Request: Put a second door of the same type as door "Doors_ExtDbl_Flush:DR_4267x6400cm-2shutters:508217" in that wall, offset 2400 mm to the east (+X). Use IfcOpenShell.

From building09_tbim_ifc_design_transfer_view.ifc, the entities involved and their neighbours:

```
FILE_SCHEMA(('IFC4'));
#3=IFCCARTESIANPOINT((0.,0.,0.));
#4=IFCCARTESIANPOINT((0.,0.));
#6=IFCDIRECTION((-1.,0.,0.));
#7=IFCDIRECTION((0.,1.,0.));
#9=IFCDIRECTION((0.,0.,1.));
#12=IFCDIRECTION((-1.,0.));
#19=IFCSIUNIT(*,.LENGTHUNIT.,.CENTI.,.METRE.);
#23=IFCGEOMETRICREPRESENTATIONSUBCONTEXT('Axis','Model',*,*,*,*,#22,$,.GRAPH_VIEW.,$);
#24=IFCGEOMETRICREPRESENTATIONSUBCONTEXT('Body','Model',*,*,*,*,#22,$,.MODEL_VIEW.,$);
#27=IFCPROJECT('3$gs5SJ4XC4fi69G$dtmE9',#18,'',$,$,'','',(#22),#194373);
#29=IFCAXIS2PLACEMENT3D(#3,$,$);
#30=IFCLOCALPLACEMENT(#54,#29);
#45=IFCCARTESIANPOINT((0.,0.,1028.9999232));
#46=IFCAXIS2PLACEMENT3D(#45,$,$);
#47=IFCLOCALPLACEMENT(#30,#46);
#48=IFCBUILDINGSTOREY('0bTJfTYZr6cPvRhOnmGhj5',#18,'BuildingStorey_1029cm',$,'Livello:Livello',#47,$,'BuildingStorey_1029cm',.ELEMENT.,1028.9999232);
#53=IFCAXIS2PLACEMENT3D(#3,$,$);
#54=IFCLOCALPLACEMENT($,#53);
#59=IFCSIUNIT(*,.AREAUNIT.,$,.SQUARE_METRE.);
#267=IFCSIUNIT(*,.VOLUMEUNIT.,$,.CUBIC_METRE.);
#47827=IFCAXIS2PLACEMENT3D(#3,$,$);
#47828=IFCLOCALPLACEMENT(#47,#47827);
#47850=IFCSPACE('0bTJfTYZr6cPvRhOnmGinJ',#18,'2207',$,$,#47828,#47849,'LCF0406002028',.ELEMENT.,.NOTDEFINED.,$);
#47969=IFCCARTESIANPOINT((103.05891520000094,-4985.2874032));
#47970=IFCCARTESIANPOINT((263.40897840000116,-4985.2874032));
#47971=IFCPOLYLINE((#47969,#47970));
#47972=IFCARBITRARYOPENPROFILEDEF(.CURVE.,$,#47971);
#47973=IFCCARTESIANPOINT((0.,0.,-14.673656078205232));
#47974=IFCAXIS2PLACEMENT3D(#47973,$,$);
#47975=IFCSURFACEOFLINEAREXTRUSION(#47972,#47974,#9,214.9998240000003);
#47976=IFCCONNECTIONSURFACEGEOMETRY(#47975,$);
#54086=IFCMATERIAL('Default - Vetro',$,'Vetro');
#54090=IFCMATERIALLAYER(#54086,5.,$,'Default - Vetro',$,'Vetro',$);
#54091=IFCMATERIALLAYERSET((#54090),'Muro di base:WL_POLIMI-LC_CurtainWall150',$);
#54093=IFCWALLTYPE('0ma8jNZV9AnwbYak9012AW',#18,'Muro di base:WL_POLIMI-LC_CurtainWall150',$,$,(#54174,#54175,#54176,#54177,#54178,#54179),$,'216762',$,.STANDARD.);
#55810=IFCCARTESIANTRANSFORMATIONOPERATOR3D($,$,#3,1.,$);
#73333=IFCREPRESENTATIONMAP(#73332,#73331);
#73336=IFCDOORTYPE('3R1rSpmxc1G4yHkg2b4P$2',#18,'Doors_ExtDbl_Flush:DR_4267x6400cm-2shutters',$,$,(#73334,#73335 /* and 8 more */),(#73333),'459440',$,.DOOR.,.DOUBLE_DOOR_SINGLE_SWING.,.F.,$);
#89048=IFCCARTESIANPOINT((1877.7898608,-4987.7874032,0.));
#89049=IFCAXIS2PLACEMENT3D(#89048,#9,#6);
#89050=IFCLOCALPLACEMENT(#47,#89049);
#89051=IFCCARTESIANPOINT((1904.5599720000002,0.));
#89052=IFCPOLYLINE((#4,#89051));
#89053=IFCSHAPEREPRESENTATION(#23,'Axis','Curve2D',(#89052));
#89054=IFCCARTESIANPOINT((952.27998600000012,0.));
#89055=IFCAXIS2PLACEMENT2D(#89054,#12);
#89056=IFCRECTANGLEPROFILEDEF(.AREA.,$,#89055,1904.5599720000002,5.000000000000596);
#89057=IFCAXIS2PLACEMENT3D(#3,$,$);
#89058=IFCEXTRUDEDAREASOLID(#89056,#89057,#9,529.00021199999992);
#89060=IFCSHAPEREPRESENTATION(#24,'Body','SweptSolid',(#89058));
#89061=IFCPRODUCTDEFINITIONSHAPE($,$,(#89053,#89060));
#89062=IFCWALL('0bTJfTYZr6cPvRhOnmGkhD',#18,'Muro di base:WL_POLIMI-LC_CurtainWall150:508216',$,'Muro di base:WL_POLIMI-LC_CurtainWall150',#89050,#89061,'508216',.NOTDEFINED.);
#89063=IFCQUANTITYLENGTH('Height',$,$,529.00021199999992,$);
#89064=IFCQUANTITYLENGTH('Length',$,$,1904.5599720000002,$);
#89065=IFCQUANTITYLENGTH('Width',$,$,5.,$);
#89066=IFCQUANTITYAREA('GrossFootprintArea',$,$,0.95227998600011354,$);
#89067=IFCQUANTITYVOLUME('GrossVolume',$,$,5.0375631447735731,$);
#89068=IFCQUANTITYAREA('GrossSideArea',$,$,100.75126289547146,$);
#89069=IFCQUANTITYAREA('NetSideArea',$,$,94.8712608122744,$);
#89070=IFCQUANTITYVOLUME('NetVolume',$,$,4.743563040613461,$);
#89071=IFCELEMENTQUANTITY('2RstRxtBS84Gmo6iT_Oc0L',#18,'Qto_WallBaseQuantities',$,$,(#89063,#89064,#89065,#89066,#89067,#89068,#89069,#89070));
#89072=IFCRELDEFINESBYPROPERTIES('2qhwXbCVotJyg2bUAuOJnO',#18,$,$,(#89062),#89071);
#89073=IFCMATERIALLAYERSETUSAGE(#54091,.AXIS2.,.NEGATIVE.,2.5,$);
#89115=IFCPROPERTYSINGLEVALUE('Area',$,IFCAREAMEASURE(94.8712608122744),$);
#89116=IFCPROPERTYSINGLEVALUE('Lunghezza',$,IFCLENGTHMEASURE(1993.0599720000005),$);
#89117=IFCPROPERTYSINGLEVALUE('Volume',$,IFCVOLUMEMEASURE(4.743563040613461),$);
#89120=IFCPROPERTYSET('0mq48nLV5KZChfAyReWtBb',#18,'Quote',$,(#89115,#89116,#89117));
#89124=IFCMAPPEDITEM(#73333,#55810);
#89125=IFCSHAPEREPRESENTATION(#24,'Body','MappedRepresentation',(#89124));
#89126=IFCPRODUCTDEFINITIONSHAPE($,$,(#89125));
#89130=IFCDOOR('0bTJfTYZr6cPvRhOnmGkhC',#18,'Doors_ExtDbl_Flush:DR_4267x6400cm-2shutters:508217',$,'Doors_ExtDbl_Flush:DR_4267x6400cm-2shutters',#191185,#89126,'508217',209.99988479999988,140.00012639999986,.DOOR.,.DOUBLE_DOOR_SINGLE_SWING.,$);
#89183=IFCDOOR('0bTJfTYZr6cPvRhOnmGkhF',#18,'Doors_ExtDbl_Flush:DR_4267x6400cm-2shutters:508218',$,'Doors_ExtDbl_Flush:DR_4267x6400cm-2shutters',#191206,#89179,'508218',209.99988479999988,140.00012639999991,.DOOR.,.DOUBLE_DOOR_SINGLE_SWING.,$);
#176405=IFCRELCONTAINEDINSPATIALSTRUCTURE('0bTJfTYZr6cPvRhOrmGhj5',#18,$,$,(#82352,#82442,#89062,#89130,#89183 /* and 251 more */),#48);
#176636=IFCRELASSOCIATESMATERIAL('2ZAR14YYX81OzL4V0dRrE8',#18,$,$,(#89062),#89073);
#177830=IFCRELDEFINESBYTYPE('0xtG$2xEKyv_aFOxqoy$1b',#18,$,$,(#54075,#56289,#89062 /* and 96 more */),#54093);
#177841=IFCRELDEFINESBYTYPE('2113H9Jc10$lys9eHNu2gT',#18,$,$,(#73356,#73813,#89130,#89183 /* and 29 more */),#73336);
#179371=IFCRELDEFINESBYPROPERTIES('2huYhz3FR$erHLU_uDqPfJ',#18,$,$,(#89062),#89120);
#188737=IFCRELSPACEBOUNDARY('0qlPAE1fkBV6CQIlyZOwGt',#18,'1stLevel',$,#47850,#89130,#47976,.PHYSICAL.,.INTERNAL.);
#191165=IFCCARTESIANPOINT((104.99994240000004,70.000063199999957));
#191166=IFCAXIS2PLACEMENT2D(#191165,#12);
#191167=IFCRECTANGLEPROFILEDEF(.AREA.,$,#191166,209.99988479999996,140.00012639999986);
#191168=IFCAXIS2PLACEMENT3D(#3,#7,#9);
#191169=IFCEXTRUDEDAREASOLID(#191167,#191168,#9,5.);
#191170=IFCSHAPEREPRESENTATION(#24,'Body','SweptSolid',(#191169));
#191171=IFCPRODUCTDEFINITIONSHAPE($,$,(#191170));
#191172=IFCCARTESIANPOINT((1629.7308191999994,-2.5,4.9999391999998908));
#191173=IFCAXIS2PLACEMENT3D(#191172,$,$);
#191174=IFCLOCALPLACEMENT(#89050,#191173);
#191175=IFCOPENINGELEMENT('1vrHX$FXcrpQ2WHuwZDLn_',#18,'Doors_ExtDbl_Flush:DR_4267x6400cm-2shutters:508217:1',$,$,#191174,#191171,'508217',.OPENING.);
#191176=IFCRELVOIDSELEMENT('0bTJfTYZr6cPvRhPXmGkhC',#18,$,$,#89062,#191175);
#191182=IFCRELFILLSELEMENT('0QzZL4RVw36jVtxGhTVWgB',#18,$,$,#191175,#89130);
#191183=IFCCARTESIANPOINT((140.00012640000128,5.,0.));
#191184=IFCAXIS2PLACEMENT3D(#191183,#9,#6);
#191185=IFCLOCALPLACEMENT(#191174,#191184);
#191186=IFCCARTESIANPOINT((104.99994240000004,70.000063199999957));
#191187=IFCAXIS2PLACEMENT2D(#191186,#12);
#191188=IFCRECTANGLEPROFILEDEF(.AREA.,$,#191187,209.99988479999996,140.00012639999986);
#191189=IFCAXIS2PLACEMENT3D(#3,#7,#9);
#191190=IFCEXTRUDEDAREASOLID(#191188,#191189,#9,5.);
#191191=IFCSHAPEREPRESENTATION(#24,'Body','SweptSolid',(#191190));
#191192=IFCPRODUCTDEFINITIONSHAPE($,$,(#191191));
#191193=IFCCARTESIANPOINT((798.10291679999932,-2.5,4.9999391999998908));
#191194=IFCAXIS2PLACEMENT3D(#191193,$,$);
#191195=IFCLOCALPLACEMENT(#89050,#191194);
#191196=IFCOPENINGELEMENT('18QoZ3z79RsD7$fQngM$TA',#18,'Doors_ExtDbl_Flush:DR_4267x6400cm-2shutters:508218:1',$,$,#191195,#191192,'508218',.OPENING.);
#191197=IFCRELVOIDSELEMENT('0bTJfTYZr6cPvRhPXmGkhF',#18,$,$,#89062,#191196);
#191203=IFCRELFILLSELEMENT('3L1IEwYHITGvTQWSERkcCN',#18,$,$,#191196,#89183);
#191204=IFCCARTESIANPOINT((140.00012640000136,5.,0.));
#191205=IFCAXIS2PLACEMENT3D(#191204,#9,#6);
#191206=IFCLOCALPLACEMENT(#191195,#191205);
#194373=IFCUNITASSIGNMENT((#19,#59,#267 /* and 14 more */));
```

```python
import numpy as np
import ifcopenshell
import ifcopenshell.api.feature
import ifcopenshell.api.geometry
import ifcopenshell.api.pset
import ifcopenshell.api.root
import ifcopenshell.geom
import ifcopenshell.util.element
import ifcopenshell.util.placement
import ifcopenshell.util.shape
import ifcopenshell.util.unit

model = ifcopenshell.open("building09_tbim_ifc_design_transfer_view.ifc")
unit_scale = ifcopenshell.util.unit.calculate_unit_scale(model)
area_scale = ifcopenshell.util.unit.calculate_unit_scale(model, "AREAUNIT")
volume_scale = ifcopenshell.util.unit.calculate_unit_scale(model, "VOLUMEUNIT")
settings = ifcopenshell.geom.settings()


def volume(element):
    """Net volume in cubic metres, openings subtracted."""
    shape = ifcopenshell.geom.create_shape(settings, element)
    return ifcopenshell.util.shape.get_volume(shape.geometry)


def reuse_history(source, copy):
    """copy_class also copies each property set's owner history, people and application; keep the originals."""
    for rel in copy.IsDefinedBy:
        if rel.is_a("IfcRelDefinesByProperties") and (history := rel.RelatingPropertyDefinition.OwnerHistory):
            rel.RelatingPropertyDefinition.OwnerHistory = source.OwnerHistory
            ifcopenshell.util.element.remove_deep2(model, history)


door = model.by_id(89130)
opening = door.FillsVoids[0].RelatingOpeningElement
wall = opening.VoidsElements[0].RelatingBuildingElement
before = volume(wall)
shift = ifcopenshell.util.placement.get_local_placement(wall.ObjectPlacement)[:3, 0] * -2.4 / unit_scale

# copy_class copies the void relationship, type, container and properties, but no geometry.
new_opening = ifcopenshell.api.root.copy_class(model, product=opening)
new_opening.Representation = ifcopenshell.util.element.copy_deep(
    model, opening.Representation, exclude=["IfcGeometricRepresentationContext", "IfcRepresentationMap"]
)
new_opening.Name = "Doors_ExtDbl_Flush:DR_4267x6400cm-2shutters"
new_opening.Tag = None
reuse_history(opening, new_opening)
new_door = ifcopenshell.api.root.copy_class(model, product=door)
new_door.Representation = ifcopenshell.util.element.copy_deep(
    model, door.Representation, exclude=["IfcGeometricRepresentationContext", "IfcRepresentationMap"]
)
new_door.Name = "Doors_ExtDbl_Flush:DR_4267x6400cm-2shutters"
new_door.Tag = None
reuse_history(door, new_door)
ifcopenshell.api.feature.add_filling(model, opening=new_opening, element=new_door)

for old, new in ((opening, new_opening), (door, new_door)):
    matrix = ifcopenshell.util.placement.get_local_placement(old.ObjectPlacement)
    matrix[:3, 3] += shift
    ifcopenshell.api.geometry.edit_object_placement(model, product=new, matrix=matrix, is_si=False)

# The copied space boundaries still share their surfaces with the original.
for rel in new_door.ProvidesBoundaries:
    if rel.ConnectionGeometry:
        rel.ConnectionGeometry = ifcopenshell.util.element.copy_deep(model, rel.ConnectionGeometry)

# Space boundary surfaces are stored in each space's coordinates; move them too.
for rel in new_door.ProvidesBoundaries:
    if not rel.ConnectionGeometry:
        continue
    surface = rel.ConnectionGeometry.SurfaceOnRelatingElement
    space_matrix = ifcopenshell.util.placement.get_local_placement(rel.RelatingSpace.ObjectPlacement)
    point = np.array(surface.Position.Location.Coordinates) + space_matrix[:3, :3].T @ shift
    surface.Position = model.createIfcAxis2Placement3D(
        model.createIfcCartesianPoint(point.tolist()), surface.Position.Axis, surface.Position.RefDirection
    )

after = volume(wall)
thickness = 0.05  # wall thickness in metres

# Update the wall's stored quantities.
qto = model.by_id(ifcopenshell.util.element.get_pset(wall, "Qto_WallBaseQuantities", should_inherit=False)["id"])
ifcopenshell.api.pset.edit_qto(model, qto=qto, properties={
    "NetSideArea": after / thickness / area_scale,
    "NetVolume": after / volume_scale,
})
pset = model.by_id(ifcopenshell.util.element.get_pset(wall, "Quote", should_inherit=False)["id"])
ifcopenshell.api.pset.edit_pset(model, pset=pset, properties={
    "Area": model.create_entity("IfcAreaMeasure", after / thickness / area_scale),
    "Volume": model.create_entity("IfcVolumeMeasure", after / volume_scale),
})

print(f"wall volume {before:.3f} -> {after:.3f} m3")

model.write("building09_tbim_ifc_design_transfer_view_rev.ifc")
```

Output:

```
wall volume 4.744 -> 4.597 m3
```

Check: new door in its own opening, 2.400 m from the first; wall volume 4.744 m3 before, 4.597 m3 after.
